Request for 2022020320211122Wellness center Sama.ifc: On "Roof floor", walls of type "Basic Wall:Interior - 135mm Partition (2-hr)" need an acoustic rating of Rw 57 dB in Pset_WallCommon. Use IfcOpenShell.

First a look at what the model holds.

```python
import ifcopenshell
import ifcopenshell.util.element

model = ifcopenshell.open("2022020320211122Wellness center Sama.ifc")
print(model.schema)
storey = next(s for s in model.by_type("IfcBuildingStorey") if s.Name == "Roof floor")
walls = [e for e in ifcopenshell.util.element.get_decomposition(storey) if e.is_a("IfcWall")]
seen = {}
for e in walls:
    element_type = ifcopenshell.util.element.get_type(e)
    key = (element_type.Name if element_type != e and element_type else None, ifcopenshell.util.element.get_pset(e, "Pset_WallCommon", "AcousticRating"))
    seen[key] = seen.get(key, 0) + 1
for (name, value), count in sorted(seen.items(), key=str):
    print(count, "x", name, "|", value)
```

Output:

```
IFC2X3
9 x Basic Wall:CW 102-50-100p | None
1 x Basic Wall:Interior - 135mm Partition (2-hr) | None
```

```python
import ifcopenshell
import ifcopenshell.api.pset
import ifcopenshell.util.element

model = ifcopenshell.open("2022020320211122Wellness center Sama.ifc")

storey = next(s for s in model.by_type("IfcBuildingStorey") if s.Name == "Roof floor")
walls = [e for e in ifcopenshell.util.element.get_decomposition(storey) if e.is_a("IfcWall")]

count = 0
for e in walls:
    element_type = ifcopenshell.util.element.get_type(e)
    if element_type in (None, e) or element_type.Name != "Basic Wall:Interior - 135mm Partition (2-hr)":
        continue
    # add_pset returns the element's existing set when there is one.
    pset = ifcopenshell.api.pset.add_pset(model, product=e, name="Pset_WallCommon")
    ifcopenshell.api.pset.edit_pset(model, pset=pset, properties={"AcousticRating": "Rw 57 dB"})
    count += 1

print(count, "walls updated")

model.write("2022020320211122Wellness center Sama_rev.ifc")
```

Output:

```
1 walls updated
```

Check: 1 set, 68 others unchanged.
